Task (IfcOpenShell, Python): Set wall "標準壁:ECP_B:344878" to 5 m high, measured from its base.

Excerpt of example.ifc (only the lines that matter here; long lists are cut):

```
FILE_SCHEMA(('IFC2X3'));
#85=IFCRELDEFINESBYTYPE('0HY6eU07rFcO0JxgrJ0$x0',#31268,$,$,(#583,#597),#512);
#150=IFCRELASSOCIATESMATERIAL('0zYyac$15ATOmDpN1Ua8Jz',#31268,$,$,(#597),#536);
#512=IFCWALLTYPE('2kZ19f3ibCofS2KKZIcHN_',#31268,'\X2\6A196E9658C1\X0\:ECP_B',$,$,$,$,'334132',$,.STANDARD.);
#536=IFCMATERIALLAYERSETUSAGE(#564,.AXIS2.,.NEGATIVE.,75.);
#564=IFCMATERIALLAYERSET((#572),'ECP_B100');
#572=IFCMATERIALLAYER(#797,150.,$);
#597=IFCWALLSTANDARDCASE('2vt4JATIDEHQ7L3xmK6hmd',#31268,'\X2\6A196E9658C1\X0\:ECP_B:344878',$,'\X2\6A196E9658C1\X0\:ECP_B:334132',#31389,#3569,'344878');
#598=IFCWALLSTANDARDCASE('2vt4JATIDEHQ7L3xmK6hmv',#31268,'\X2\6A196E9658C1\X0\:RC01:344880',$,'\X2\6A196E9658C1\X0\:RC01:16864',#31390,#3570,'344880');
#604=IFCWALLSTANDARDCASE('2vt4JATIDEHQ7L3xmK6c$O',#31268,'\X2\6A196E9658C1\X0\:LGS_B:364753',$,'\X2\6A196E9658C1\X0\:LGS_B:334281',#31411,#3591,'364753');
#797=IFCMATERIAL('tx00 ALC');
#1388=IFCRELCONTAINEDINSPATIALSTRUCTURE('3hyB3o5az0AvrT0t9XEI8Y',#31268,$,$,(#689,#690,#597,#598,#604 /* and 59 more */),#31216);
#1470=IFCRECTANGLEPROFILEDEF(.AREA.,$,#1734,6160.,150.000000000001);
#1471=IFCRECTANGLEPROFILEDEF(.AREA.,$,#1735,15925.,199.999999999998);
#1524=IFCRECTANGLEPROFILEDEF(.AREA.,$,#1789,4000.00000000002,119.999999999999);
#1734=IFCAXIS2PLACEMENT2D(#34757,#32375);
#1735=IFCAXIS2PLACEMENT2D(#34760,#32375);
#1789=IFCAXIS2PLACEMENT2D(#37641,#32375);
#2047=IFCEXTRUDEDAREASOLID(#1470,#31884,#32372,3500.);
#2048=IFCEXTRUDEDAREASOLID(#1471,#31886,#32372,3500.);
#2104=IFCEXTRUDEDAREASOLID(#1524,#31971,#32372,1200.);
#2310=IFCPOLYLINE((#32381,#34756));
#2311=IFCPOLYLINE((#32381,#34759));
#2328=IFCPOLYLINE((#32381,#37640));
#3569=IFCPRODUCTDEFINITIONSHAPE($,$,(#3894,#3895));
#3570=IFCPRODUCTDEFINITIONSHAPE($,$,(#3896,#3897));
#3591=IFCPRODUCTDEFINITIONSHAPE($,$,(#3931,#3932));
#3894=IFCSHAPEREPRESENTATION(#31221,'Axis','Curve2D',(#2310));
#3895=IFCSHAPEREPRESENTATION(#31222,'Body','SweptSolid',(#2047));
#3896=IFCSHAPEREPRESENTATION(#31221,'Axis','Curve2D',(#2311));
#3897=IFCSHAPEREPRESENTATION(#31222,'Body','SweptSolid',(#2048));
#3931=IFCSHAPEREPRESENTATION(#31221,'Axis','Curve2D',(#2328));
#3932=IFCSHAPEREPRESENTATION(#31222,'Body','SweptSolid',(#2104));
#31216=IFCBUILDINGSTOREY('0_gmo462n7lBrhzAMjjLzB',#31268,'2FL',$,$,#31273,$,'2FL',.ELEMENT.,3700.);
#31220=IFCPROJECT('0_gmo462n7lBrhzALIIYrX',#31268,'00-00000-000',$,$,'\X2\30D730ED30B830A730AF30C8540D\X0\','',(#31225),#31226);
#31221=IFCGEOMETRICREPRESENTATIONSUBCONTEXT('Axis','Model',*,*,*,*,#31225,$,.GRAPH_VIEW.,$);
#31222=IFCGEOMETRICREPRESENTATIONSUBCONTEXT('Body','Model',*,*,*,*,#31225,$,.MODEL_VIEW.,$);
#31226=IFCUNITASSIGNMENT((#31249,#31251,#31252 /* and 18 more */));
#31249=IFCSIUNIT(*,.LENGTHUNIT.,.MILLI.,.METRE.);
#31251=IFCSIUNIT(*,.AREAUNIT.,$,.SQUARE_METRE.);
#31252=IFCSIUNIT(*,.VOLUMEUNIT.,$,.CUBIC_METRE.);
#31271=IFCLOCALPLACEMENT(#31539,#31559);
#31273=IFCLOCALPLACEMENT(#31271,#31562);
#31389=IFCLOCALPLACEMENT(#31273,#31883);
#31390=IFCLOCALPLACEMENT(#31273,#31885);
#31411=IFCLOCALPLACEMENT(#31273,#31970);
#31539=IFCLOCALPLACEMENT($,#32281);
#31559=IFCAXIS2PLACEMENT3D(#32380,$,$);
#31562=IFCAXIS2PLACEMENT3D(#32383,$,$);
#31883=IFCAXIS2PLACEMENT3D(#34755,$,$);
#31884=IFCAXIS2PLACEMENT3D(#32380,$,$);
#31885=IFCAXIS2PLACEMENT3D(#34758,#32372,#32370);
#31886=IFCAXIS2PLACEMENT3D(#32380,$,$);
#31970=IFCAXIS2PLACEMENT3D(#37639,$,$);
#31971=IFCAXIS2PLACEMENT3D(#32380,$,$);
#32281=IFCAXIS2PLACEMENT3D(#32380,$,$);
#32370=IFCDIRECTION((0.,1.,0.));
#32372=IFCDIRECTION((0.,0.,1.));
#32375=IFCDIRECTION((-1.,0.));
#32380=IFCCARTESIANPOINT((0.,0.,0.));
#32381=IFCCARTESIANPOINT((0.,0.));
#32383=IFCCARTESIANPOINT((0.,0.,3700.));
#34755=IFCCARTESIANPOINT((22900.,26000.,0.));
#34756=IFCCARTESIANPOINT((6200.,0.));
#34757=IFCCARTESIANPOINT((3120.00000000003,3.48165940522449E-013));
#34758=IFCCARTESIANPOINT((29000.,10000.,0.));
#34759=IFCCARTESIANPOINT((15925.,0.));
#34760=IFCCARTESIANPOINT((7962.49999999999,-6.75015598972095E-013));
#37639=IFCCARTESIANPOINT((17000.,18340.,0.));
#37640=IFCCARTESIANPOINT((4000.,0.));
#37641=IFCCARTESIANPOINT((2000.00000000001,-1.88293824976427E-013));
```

```python
import ifcopenshell
import ifcopenshell.geom
import ifcopenshell.util.representation
import ifcopenshell.util.shape

model = ifcopenshell.open("example.ifc")
settings = ifcopenshell.geom.settings()


def volume(element):
    """Net volume in cubic metres, openings subtracted."""
    shape = ifcopenshell.geom.create_shape(settings, element)
    return ifcopenshell.util.shape.get_volume(shape.geometry)


wall = model.by_guid("2vt4JATIDEHQ7L3xmK6hmd")
before = volume(wall)

body = ifcopenshell.util.representation.get_representation(wall, "Model", "Body")
solid = body.Items[0]
old_height = solid.Depth
solid.Depth = 5000.0
after = volume(wall)

print(f"height {old_height:g} -> {solid.Depth:g}, volume {before:.3f} -> {after:.3f} m3")

model.write("example_updated.ifc")
```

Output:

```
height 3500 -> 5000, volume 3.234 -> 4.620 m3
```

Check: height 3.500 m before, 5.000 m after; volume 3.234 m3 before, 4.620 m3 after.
